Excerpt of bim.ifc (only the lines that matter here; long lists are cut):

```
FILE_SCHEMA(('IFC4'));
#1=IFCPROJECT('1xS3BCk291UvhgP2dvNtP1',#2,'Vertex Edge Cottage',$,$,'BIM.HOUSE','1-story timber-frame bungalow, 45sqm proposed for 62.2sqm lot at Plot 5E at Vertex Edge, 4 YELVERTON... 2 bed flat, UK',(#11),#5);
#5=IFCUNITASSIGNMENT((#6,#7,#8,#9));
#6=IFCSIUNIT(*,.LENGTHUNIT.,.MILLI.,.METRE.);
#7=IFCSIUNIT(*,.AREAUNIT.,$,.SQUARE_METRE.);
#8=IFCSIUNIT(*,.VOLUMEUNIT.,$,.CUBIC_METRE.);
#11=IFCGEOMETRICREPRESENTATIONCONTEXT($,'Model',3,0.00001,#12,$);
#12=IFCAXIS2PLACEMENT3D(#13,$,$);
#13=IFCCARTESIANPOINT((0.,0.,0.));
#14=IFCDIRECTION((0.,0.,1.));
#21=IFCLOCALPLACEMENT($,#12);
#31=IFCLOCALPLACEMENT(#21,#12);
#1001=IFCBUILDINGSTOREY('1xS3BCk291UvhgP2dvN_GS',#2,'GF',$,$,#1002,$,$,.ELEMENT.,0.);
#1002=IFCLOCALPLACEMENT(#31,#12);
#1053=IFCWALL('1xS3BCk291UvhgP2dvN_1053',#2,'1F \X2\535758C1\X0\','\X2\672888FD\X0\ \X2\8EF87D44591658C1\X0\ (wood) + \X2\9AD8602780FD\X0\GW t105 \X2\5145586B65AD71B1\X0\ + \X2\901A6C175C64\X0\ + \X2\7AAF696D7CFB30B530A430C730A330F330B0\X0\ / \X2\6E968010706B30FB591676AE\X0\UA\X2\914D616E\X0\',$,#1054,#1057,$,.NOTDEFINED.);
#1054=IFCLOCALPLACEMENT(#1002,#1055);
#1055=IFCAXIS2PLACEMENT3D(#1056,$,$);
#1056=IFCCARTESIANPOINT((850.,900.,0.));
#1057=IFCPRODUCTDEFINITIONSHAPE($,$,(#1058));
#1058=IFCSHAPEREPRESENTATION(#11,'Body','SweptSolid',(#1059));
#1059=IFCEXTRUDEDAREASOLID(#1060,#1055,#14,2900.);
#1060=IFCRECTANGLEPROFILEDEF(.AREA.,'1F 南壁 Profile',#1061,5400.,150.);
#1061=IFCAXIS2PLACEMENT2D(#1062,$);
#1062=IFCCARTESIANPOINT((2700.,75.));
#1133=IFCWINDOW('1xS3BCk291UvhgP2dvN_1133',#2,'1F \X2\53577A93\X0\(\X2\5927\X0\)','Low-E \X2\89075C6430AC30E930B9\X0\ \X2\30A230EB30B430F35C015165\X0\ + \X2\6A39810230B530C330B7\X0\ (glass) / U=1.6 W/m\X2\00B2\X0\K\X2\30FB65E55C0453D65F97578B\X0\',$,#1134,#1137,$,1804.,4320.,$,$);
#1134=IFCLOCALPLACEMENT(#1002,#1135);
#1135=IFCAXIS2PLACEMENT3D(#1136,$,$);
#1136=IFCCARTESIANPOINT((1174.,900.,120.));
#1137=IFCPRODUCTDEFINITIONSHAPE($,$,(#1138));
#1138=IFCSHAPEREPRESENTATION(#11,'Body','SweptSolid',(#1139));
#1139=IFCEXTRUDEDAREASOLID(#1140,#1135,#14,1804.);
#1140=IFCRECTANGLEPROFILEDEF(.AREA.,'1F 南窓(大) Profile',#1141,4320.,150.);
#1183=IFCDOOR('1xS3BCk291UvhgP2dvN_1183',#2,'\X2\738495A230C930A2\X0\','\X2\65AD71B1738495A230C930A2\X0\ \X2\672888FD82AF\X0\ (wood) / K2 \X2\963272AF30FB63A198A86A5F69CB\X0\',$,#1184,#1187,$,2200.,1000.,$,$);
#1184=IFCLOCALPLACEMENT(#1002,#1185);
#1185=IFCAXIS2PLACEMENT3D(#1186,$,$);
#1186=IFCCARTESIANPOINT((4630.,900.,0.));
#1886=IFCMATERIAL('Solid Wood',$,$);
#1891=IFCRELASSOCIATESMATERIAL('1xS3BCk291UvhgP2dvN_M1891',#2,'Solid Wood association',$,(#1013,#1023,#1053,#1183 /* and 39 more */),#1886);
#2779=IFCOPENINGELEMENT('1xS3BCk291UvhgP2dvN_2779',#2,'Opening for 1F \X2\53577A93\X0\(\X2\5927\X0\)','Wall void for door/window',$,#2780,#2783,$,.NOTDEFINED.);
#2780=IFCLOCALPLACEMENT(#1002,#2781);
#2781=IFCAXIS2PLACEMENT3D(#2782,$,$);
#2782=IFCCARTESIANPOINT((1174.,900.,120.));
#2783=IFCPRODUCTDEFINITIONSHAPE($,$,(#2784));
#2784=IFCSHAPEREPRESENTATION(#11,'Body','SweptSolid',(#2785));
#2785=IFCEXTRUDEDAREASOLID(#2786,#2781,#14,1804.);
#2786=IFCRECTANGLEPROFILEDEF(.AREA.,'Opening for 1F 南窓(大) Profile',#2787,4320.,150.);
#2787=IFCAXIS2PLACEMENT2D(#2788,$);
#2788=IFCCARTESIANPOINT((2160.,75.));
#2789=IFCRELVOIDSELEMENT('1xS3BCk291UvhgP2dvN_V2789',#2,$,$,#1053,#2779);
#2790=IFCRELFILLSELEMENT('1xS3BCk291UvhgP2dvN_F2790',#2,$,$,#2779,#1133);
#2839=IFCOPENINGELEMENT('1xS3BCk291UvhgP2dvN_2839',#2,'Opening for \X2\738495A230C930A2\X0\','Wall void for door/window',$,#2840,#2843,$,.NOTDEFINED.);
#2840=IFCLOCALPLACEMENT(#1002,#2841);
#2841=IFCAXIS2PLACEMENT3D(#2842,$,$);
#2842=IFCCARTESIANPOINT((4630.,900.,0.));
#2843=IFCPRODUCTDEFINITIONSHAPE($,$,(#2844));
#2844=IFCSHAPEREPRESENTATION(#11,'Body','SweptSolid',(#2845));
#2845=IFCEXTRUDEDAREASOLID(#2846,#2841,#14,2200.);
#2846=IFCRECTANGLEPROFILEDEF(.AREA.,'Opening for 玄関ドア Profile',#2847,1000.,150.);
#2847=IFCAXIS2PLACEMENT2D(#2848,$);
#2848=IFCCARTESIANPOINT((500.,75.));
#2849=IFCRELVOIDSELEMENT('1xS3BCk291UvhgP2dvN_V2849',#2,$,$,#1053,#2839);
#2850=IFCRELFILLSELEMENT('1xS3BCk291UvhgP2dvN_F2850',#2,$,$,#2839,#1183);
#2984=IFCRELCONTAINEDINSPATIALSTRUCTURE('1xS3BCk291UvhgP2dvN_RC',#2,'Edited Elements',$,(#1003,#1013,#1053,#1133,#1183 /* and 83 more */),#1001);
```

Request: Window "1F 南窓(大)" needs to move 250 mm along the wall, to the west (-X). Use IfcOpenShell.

```python
import ifcopenshell
import ifcopenshell.api.geometry
import ifcopenshell.util.placement

model = ifcopenshell.open("bim.ifc")

window = model.by_id(1133)
opening = window.FillsVoids[0].RelatingOpeningElement
wall = opening.VoidsElements[0].RelatingBuildingElement

wall_matrix = ifcopenshell.util.placement.get_local_placement(wall.ObjectPlacement)
shift = wall_matrix[:3, 0] * -250.0
before = ifcopenshell.util.placement.get_local_placement(window.ObjectPlacement)[:3, 3].copy()

# The window is not placed relative to its opening, so move both.
for product in (opening, window):
    matrix = ifcopenshell.util.placement.get_local_placement(product.ObjectPlacement)
    matrix[:3, 3] += shift
    ifcopenshell.api.geometry.edit_object_placement(model, product=product, matrix=matrix, is_si=False)

after = ifcopenshell.util.placement.get_local_placement(window.ObjectPlacement)[:3, 3]
print("window moved by", (after - before).round(3) + 0.0)

model.write("bim_updated.ifc")
```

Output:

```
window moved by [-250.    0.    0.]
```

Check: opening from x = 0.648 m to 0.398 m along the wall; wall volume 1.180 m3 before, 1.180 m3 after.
